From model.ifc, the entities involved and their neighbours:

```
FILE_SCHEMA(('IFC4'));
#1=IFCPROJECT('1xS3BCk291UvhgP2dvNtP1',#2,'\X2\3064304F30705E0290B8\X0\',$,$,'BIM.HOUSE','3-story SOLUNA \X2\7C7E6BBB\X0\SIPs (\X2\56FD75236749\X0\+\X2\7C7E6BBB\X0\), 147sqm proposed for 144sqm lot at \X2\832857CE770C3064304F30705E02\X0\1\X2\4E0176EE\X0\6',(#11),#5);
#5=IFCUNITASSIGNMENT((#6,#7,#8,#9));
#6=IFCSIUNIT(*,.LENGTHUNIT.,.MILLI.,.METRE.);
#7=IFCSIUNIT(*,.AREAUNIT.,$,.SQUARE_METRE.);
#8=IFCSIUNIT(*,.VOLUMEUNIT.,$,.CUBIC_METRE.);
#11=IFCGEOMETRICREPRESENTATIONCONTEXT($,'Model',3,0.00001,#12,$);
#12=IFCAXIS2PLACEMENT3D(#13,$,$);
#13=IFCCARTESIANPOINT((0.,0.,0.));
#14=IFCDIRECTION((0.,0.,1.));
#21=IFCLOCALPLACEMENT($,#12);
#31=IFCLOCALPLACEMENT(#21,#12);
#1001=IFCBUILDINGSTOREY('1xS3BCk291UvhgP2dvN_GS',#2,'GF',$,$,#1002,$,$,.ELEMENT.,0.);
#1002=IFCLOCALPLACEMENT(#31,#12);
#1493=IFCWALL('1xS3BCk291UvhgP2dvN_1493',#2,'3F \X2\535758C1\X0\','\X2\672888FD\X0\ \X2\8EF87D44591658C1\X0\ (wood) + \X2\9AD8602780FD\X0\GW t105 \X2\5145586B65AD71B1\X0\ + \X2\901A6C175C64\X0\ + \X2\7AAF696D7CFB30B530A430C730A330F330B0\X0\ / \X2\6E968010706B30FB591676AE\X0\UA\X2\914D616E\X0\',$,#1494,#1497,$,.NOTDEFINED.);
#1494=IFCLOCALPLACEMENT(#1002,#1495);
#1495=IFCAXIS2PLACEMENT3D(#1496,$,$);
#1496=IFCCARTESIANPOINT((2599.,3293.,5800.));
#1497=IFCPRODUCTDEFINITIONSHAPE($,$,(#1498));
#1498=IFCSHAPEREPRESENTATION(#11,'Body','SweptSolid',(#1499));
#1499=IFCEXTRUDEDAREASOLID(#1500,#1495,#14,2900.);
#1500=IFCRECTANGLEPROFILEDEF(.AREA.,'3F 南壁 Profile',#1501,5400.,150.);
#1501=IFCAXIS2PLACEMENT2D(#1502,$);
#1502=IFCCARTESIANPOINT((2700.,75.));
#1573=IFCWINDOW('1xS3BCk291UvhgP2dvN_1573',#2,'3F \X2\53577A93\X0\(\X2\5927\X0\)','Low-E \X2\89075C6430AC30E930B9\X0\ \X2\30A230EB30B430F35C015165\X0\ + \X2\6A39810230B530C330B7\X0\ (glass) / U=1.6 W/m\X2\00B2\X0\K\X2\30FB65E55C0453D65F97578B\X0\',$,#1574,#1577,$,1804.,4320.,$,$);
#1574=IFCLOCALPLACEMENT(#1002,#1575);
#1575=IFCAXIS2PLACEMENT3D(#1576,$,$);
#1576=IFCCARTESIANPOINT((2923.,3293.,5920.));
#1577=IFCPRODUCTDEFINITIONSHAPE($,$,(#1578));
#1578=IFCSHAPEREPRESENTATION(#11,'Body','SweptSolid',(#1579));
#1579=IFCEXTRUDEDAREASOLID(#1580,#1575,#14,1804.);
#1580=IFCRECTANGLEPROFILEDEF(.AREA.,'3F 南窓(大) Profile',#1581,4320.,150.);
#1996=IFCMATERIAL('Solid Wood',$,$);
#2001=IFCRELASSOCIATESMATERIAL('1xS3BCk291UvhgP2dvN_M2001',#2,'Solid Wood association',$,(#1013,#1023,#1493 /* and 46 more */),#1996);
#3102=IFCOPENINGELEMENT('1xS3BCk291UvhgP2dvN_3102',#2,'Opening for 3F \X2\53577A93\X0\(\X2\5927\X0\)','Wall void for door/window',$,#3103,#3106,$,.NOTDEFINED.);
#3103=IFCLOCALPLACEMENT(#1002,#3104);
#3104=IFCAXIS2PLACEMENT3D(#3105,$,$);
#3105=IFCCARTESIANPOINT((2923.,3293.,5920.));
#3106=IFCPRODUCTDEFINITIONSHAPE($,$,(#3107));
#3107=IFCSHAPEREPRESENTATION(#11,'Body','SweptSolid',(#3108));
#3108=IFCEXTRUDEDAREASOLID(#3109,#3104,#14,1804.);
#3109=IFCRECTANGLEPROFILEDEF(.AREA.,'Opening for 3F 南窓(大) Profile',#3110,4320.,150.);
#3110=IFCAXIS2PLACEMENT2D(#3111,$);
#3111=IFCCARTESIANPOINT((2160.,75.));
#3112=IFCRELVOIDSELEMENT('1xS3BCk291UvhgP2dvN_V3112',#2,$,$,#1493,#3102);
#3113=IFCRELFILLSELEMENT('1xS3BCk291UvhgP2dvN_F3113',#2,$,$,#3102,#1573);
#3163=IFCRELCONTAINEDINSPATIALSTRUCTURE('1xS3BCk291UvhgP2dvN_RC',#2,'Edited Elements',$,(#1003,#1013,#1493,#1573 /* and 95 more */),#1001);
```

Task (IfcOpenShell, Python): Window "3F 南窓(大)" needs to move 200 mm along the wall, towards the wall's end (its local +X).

```python
import ifcopenshell
import ifcopenshell.api.geometry
import ifcopenshell.util.placement
import ifcopenshell.util.unit

model = ifcopenshell.open("model.ifc")
unit_scale = ifcopenshell.util.unit.calculate_unit_scale(model)

window = model.by_id(1573)
opening = window.FillsVoids[0].RelatingOpeningElement
wall = opening.VoidsElements[0].RelatingBuildingElement

wall_matrix = ifcopenshell.util.placement.get_local_placement(wall.ObjectPlacement)
shift = wall_matrix[:3, 0] * 0.2 / unit_scale
before = ifcopenshell.util.placement.get_local_placement(window.ObjectPlacement)[:3, 3].copy()

# The window is not placed relative to its opening, so move both.
for product in (opening, window):
    matrix = ifcopenshell.util.placement.get_local_placement(product.ObjectPlacement)
    matrix[:3, 3] += shift
    ifcopenshell.api.geometry.edit_object_placement(model, product=product, matrix=matrix, is_si=False)

after = ifcopenshell.util.placement.get_local_placement(window.ObjectPlacement)[:3, 3]
print("window moved by", (after - before).round(3) + 0.0)

model.write("model_edited.ifc")
```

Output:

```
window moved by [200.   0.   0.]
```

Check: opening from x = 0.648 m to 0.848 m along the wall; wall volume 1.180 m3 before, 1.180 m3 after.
